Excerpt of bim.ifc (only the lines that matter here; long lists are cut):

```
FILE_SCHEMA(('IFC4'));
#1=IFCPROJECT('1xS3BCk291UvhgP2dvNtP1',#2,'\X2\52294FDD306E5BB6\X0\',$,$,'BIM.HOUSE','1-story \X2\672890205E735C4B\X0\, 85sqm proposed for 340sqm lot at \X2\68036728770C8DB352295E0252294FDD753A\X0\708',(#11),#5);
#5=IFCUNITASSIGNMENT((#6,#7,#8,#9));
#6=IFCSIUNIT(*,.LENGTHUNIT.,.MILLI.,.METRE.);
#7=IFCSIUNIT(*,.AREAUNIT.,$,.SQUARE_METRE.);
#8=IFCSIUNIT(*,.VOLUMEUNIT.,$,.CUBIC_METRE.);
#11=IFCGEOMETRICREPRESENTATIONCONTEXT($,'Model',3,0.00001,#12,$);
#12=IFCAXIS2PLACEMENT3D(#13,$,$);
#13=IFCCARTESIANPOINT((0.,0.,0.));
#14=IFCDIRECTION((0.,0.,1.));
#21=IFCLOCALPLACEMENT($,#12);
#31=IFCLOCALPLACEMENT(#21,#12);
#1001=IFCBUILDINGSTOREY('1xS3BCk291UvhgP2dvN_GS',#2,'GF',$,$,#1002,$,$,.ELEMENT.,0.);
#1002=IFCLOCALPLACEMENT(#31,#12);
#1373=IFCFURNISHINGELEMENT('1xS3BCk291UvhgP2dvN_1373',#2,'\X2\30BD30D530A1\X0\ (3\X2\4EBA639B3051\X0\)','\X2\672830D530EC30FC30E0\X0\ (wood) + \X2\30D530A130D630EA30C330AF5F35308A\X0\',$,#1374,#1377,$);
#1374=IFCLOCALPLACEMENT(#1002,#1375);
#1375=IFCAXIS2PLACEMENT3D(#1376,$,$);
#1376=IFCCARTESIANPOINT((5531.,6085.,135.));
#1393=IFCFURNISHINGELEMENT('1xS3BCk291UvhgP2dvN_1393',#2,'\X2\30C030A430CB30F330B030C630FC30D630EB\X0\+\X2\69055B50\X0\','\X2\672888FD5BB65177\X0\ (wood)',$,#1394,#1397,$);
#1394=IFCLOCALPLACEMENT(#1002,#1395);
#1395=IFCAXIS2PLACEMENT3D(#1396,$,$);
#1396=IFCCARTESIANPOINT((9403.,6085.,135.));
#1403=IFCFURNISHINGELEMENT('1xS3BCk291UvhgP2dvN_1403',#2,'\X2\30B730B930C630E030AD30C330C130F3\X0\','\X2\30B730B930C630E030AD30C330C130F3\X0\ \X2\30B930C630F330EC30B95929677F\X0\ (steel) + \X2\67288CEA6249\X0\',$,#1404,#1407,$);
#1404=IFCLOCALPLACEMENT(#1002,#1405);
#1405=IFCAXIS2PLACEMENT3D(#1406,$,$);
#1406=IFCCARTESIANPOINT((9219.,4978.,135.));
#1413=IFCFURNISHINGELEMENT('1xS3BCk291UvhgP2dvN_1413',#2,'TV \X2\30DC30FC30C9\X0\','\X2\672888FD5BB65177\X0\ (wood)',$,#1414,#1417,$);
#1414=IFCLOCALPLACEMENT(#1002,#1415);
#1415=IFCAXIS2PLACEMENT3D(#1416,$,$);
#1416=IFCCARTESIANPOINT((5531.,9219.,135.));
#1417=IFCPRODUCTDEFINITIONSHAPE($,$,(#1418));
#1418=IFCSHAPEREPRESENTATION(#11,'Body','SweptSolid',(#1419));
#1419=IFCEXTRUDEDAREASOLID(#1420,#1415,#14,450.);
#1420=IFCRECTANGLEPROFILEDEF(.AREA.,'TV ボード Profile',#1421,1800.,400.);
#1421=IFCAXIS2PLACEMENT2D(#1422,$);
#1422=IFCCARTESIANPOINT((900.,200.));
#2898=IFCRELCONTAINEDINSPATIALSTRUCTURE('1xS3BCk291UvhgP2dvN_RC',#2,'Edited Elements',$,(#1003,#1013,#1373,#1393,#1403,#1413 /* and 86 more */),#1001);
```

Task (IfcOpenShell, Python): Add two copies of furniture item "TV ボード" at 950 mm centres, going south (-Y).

```python
import numpy as np
import ifcopenshell
import ifcopenshell.api.geometry
import ifcopenshell.api.root
import ifcopenshell.util.element
import ifcopenshell.util.placement
import ifcopenshell.util.unit

model = ifcopenshell.open("bim.ifc")
unit_scale = ifcopenshell.util.unit.calculate_unit_scale(model)


def reuse_history(source, copy):
    """copy_class also copies each property set's owner history, people and application; keep the originals."""
    for rel in copy.IsDefinedBy:
        if rel.is_a("IfcRelDefinesByProperties") and (history := rel.RelatingPropertyDefinition.OwnerHistory):
            rel.RelatingPropertyDefinition.OwnerHistory = source.OwnerHistory
            ifcopenshell.util.element.remove_deep2(model, history)


source = model.by_id(1413)
base = ifcopenshell.util.placement.get_local_placement(source.ObjectPlacement)
step = np.array([0.0, -1.0, 0.0]) * 0.95 / unit_scale

for i in range(1, 3):
    copy = ifcopenshell.api.root.copy_class(model, product=source)
    copy.Representation = ifcopenshell.util.element.copy_deep(
        model, source.Representation, exclude=["IfcGeometricRepresentationContext", "IfcRepresentationMap"]
    )
    reuse_history(source, copy)
    matrix = base.copy()
    matrix[:3, 3] += i * step
    print("added at", matrix[:3, 3].round(3) + 0.0)
    ifcopenshell.api.geometry.edit_object_placement(model, product=copy, matrix=matrix, is_si=False)

model.write("bim_updated.ifc")
```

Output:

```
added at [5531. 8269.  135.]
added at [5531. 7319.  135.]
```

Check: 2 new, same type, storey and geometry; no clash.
